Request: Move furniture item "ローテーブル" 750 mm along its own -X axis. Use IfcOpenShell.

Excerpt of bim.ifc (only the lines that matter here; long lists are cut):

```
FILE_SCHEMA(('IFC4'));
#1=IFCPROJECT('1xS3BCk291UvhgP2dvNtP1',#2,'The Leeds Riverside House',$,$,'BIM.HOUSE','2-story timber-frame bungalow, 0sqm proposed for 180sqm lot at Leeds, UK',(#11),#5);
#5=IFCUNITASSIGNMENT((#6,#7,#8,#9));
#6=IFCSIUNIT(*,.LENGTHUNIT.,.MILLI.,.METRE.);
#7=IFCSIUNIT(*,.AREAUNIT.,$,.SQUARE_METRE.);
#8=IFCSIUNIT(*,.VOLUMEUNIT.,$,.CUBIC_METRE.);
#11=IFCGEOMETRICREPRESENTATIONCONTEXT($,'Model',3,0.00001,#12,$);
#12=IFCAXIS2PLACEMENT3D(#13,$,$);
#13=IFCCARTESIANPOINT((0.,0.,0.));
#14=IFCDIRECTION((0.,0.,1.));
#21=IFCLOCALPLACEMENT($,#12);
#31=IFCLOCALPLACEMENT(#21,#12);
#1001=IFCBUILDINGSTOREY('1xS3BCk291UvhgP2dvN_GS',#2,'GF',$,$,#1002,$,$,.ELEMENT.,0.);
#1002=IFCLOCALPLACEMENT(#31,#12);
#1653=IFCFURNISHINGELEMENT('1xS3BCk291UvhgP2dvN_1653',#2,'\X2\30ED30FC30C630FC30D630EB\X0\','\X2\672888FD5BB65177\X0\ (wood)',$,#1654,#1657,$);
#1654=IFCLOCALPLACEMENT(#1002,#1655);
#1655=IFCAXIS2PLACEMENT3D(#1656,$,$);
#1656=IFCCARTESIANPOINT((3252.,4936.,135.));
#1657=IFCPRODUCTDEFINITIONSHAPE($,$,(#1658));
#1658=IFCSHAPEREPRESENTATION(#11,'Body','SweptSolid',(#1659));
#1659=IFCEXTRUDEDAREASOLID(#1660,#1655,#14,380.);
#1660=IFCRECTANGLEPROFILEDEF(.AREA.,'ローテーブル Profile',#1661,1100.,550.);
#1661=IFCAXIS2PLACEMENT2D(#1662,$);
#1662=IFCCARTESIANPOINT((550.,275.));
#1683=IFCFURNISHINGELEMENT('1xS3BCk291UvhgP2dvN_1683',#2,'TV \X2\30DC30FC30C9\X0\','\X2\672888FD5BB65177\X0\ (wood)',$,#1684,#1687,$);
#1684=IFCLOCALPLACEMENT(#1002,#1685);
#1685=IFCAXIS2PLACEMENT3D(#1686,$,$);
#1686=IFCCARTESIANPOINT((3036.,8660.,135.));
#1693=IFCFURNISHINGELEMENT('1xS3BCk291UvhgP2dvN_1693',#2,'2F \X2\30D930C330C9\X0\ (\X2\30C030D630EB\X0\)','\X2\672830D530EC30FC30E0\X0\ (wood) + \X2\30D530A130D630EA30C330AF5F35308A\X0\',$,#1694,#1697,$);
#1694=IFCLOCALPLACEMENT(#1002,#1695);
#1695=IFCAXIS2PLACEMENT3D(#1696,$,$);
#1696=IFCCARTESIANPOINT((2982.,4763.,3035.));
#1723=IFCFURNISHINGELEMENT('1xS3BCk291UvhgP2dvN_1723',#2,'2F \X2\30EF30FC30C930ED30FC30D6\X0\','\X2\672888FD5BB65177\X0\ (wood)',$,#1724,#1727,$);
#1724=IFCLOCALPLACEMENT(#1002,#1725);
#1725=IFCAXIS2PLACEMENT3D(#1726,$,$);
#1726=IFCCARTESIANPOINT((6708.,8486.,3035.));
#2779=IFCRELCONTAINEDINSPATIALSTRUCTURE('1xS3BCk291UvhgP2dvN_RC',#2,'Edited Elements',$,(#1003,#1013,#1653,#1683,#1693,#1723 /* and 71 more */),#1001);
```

```python
import ifcopenshell
import ifcopenshell.api.geometry
import ifcopenshell.util.placement

model = ifcopenshell.open("bim.ifc")

item = model.by_guid("1xS3BCk291UvhgP2dvN_1653")
matrix = ifcopenshell.util.placement.get_local_placement(item.ObjectPlacement)
matrix[:3, 3] -= matrix[:3, 0] * 750.0
ifcopenshell.api.geometry.edit_object_placement(model, product=item, matrix=matrix, is_si=False)

print(ifcopenshell.util.placement.get_local_placement(item.ObjectPlacement).round(3) + 0.0)

model.write("bim-out.ifc")
```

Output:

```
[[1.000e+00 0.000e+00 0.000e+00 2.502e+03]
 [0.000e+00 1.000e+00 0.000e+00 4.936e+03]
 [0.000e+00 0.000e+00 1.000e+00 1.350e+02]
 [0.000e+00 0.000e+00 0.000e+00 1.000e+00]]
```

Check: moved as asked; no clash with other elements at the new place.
